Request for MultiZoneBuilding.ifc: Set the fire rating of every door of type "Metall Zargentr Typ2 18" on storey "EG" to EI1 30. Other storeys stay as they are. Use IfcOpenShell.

First a look at what the model holds.

```python
import ifcopenshell
import ifcopenshell.util.element

model = ifcopenshell.open("MultiZoneBuilding.ifc")
print(model.schema)
storey = next(s for s in model.by_type("IfcBuildingStorey") if s.Name == "EG")
doors = [e for e in ifcopenshell.util.element.get_decomposition(storey) if e.is_a("IfcDoor")]
seen = {}
for e in doors:
    element_type = ifcopenshell.util.element.get_type(e)
    key = (element_type.Name if element_type != e and element_type else None, ifcopenshell.util.element.get_pset(e, "Pset_DoorCommon", "FireRating"))
    seen[key] = seen.get(key, 0) + 1
for (name, value), count in sorted(seen.items(), key=str):
    print(count, "x", name, "|", value)
```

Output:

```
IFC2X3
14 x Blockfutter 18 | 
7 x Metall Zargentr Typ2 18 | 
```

```python
import ifcopenshell
import ifcopenshell.api.pset
import ifcopenshell.util.element

model = ifcopenshell.open("MultiZoneBuilding.ifc")

storey = next(s for s in model.by_type("IfcBuildingStorey") if s.Name == "EG")
doors = [e for e in ifcopenshell.util.element.get_decomposition(storey) if e.is_a("IfcDoor")]

count = 0
for e in doors:
    element_type = ifcopenshell.util.element.get_type(e)
    if element_type in (None, e) or element_type.Name != 'Metall Zargent\x9fr Typ2 18':
        continue
    # add_pset returns the element's existing set when there is one.
    pset = ifcopenshell.api.pset.add_pset(model, product=e, name="Pset_DoorCommon")
    ifcopenshell.api.pset.edit_pset(model, pset=pset, properties={"FireRating": "EI1 30"})
    count += 1

print(count, "doors updated")

model.write("MultiZoneBuilding_edited.ifc")
```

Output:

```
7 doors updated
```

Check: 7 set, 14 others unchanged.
